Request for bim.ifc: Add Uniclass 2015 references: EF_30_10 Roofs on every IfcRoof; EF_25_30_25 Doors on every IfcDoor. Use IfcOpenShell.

First a look at what the model holds.

```python
import ifcopenshell

model = ifcopenshell.open("bim.ifc")
print(model.schema)
print("classifications:", [c.Name for c in model.by_type("IfcClassification")])
for ifc_class in ("IfcDoor", "IfcRoof", "IfcStair", "IfcWall", "IfcWindow"):
    print(ifc_class, len(model.by_type(ifc_class)))
```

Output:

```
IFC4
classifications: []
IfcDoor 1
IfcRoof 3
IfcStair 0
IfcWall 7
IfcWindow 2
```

```python
import ifcopenshell
import ifcopenshell.api.classification

model = ifcopenshell.open("bim.ifc")

system = ifcopenshell.api.classification.add_classification(model, classification="Uniclass 2015")

codes = {
    "IfcRoof": ("EF_30_10", "Roofs"),
    "IfcDoor": ("EF_25_30_25", "Doors"),
}
for ifc_class, (code, name) in codes.items():
    products = model.by_type(ifc_class)
    ifcopenshell.api.classification.add_reference(
        model, products=products, classification=system, identification=code, name=name
    )
    print(code, len(products))

model.write("bim-out.ifc")
```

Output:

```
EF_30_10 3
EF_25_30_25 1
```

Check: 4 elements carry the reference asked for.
